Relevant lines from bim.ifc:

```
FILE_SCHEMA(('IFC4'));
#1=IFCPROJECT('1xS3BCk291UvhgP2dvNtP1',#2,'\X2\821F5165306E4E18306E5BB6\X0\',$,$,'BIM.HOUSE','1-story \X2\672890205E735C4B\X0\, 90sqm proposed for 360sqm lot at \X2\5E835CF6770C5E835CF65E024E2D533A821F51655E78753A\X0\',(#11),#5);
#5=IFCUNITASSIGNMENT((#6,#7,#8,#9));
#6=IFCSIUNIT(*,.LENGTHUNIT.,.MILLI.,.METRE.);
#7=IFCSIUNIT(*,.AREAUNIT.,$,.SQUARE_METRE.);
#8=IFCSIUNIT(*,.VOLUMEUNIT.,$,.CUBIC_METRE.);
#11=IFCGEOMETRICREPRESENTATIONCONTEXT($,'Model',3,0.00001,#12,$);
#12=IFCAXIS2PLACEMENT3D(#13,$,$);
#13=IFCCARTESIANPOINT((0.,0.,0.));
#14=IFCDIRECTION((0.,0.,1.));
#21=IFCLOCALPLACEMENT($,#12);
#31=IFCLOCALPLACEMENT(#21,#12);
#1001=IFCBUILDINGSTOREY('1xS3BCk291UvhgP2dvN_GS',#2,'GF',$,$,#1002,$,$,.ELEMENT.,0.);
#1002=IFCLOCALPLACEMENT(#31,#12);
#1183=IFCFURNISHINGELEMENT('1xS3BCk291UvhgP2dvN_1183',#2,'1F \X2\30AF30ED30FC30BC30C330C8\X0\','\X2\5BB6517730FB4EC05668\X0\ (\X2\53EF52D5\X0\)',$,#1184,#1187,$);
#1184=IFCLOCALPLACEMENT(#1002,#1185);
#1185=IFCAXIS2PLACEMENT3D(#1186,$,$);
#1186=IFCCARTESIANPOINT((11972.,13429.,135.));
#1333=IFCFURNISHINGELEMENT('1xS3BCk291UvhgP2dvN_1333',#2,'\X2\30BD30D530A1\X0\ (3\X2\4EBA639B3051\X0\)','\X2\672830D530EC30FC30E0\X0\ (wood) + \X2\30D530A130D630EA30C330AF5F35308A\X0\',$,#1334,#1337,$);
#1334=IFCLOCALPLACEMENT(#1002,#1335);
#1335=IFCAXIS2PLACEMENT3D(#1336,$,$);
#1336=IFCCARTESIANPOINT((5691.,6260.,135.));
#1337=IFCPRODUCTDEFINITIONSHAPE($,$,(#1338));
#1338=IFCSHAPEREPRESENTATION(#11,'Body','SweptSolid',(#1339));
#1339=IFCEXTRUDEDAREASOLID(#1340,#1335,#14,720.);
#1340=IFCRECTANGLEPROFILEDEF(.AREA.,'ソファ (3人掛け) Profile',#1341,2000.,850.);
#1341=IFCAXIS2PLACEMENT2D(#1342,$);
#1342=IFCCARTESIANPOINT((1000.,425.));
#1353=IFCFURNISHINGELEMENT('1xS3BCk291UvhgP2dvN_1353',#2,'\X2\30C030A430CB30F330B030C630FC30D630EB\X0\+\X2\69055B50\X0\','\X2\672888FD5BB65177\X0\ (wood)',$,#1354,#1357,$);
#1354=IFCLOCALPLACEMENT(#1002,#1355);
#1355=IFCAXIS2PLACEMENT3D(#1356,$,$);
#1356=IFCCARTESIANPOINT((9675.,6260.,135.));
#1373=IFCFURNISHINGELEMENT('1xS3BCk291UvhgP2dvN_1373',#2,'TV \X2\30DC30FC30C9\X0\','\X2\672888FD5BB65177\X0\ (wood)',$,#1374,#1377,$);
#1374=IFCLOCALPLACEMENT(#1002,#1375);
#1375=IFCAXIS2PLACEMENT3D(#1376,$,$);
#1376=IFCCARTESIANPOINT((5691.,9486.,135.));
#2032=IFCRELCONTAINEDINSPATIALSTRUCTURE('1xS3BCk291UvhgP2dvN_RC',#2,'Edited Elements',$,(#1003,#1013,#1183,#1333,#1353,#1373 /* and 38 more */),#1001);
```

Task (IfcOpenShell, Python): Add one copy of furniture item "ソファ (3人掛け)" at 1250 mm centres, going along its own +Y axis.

```python
import ifcopenshell
import ifcopenshell.api.geometry
import ifcopenshell.api.root
import ifcopenshell.util.element
import ifcopenshell.util.placement
import ifcopenshell.util.unit

model = ifcopenshell.open("bim.ifc")
unit_scale = ifcopenshell.util.unit.calculate_unit_scale(model)


def reuse_history(source, copy):
    """copy_class also copies each property set's owner history, people and application; keep the originals."""
    for rel in copy.IsDefinedBy:
        if rel.is_a("IfcRelDefinesByProperties") and (history := rel.RelatingPropertyDefinition.OwnerHistory):
            rel.RelatingPropertyDefinition.OwnerHistory = source.OwnerHistory
            ifcopenshell.util.element.remove_deep2(model, history)


source = model.by_guid("1xS3BCk291UvhgP2dvN_1333")
base = ifcopenshell.util.placement.get_local_placement(source.ObjectPlacement)
step = base[:3, 1] * 1.25 / unit_scale

for i in range(1, 2):
    copy = ifcopenshell.api.root.copy_class(model, product=source)
    copy.Representation = ifcopenshell.util.element.copy_deep(
        model, source.Representation, exclude=["IfcGeometricRepresentationContext", "IfcRepresentationMap"]
    )
    reuse_history(source, copy)
    matrix = base.copy()
    matrix[:3, 3] += i * step
    print("added at", matrix[:3, 3].round(3) + 0.0)
    ifcopenshell.api.geometry.edit_object_placement(model, product=copy, matrix=matrix, is_si=False)

model.write("bim_edited.ifc")
```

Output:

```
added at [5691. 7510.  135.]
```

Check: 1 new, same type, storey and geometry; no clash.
